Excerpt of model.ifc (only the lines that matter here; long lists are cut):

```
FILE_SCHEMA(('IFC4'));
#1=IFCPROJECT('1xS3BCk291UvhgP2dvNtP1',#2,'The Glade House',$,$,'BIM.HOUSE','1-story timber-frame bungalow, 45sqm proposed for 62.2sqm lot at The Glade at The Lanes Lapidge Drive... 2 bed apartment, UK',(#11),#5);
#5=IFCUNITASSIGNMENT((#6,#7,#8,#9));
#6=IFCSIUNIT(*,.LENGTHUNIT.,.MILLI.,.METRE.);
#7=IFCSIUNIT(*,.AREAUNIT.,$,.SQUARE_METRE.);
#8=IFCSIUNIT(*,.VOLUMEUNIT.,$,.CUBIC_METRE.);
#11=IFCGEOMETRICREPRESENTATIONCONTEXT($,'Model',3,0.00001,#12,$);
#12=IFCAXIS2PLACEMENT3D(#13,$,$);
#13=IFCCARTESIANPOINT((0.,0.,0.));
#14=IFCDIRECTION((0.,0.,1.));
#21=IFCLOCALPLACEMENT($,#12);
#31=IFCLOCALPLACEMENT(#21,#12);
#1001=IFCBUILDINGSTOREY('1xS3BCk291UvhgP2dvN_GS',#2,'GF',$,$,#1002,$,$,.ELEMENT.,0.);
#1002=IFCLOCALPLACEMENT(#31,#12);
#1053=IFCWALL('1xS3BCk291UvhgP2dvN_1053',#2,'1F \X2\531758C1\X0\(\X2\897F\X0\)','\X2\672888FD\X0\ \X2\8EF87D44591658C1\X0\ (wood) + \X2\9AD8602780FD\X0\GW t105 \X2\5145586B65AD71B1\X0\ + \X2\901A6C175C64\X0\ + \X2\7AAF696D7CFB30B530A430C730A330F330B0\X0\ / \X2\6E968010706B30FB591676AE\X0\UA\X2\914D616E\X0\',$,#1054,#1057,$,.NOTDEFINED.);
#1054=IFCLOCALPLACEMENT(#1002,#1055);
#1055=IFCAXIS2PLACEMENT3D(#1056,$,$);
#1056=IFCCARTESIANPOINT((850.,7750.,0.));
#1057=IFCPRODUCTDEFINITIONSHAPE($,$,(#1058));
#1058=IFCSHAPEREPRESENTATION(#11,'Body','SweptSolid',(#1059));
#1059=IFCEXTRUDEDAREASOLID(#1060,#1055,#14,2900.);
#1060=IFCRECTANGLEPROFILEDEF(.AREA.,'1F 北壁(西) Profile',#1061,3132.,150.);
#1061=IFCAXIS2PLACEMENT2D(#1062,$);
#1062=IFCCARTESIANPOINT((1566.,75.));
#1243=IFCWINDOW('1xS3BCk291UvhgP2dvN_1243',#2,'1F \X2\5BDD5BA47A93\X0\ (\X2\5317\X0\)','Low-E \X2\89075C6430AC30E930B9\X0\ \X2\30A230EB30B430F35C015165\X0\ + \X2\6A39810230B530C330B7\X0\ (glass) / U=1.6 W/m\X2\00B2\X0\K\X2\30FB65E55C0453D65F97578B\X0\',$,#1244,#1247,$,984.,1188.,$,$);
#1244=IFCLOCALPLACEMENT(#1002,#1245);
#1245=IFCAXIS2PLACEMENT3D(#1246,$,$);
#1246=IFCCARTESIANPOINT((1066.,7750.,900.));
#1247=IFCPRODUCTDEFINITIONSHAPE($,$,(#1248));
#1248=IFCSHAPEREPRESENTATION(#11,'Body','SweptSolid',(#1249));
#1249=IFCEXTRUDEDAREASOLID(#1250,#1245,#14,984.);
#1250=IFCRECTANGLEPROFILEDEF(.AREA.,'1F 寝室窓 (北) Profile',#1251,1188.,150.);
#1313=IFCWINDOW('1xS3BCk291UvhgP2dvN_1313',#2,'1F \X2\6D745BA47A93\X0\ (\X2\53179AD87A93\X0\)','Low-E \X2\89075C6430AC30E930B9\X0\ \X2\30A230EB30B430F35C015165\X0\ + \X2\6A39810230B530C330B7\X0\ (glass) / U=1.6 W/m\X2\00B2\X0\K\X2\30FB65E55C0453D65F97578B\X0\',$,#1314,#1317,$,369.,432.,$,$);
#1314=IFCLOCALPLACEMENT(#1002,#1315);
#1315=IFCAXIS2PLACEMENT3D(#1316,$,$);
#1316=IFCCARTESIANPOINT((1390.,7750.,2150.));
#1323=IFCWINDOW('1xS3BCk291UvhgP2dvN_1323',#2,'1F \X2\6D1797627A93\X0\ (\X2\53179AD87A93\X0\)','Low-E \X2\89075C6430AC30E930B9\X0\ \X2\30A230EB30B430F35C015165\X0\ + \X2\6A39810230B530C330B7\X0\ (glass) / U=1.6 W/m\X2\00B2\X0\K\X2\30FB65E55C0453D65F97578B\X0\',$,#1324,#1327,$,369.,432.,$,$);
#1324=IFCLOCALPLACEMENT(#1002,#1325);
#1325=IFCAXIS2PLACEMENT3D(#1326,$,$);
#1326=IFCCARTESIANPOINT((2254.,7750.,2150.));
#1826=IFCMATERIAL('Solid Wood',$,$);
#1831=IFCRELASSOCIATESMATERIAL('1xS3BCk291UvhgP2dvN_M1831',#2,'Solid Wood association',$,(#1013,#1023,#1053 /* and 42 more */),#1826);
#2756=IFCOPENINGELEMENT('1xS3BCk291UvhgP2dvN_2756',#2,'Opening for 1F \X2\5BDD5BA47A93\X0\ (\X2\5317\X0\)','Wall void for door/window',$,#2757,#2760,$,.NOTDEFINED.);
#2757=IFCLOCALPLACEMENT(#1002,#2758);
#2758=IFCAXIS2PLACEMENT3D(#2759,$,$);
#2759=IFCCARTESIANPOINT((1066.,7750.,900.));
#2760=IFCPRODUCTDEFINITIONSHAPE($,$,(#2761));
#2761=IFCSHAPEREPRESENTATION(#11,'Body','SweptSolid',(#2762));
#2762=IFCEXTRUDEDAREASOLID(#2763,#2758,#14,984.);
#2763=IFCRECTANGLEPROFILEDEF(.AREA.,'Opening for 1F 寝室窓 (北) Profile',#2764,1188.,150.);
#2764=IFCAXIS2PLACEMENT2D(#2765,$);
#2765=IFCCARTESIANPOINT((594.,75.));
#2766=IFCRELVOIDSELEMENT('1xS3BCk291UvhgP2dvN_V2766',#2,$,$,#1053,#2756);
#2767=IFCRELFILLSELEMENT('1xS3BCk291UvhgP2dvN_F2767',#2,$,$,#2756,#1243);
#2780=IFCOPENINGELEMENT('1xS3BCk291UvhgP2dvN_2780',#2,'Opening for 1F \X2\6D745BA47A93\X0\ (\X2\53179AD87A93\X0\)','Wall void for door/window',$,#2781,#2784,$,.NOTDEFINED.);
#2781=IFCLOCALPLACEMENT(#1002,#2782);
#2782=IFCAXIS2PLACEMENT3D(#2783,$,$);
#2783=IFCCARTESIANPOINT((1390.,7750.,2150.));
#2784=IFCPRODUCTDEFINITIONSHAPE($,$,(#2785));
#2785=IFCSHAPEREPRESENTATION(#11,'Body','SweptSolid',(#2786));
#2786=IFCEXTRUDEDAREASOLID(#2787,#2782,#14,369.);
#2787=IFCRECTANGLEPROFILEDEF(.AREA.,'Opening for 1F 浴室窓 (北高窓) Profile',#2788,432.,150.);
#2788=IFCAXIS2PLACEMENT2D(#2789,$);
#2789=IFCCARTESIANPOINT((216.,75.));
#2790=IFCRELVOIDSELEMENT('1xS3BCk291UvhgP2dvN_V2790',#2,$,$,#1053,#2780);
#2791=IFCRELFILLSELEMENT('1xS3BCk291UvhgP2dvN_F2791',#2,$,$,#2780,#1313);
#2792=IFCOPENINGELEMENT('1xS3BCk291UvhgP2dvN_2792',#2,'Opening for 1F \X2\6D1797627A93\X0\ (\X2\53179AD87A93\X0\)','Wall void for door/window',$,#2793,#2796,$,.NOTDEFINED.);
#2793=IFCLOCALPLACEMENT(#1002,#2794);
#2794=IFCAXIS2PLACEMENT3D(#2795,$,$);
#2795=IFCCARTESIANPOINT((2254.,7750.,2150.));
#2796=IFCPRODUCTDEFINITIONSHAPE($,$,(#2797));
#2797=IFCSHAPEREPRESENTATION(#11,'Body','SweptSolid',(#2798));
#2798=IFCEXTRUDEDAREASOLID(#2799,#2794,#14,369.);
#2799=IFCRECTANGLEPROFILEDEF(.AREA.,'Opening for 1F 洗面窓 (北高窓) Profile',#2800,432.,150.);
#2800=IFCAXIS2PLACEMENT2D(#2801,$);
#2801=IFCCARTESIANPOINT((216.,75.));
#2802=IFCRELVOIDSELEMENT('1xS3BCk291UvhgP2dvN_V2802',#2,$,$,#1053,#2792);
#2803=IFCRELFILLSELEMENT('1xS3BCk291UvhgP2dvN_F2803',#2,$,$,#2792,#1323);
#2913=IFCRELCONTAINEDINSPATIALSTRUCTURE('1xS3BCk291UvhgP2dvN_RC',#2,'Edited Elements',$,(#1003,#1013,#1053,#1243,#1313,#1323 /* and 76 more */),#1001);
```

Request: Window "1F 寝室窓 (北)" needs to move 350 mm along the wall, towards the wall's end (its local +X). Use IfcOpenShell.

```python
import ifcopenshell
import ifcopenshell.api.geometry
import ifcopenshell.util.placement
import ifcopenshell.util.unit

model = ifcopenshell.open("model.ifc")
unit_scale = ifcopenshell.util.unit.calculate_unit_scale(model)

window = model.by_id(1243)
opening = window.FillsVoids[0].RelatingOpeningElement
wall = opening.VoidsElements[0].RelatingBuildingElement

wall_matrix = ifcopenshell.util.placement.get_local_placement(wall.ObjectPlacement)
shift = wall_matrix[:3, 0] * 0.35 / unit_scale
before = ifcopenshell.util.placement.get_local_placement(window.ObjectPlacement)[:3, 3].copy()

# The window is not placed relative to its opening, so move both.
for product in (opening, window):
    matrix = ifcopenshell.util.placement.get_local_placement(product.ObjectPlacement)
    matrix[:3, 3] += shift
    ifcopenshell.api.geometry.edit_object_placement(model, product=product, matrix=matrix, is_si=False)

after = ifcopenshell.util.placement.get_local_placement(window.ObjectPlacement)[:3, 3]
print("window moved by", (after - before).round(3) + 0.0)

model.write("model_v2.ifc")
```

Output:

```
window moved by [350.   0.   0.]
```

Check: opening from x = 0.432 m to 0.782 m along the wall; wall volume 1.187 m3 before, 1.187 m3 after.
